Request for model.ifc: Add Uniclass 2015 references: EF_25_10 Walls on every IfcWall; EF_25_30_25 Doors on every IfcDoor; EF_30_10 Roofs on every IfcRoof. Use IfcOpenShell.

First a look at what the model holds.

```python
import ifcopenshell

model = ifcopenshell.open("model.ifc")
print(model.schema)
print("classifications:", [c.Name for c in model.by_type("IfcClassification")])
for ifc_class in ("IfcDoor", "IfcRoof", "IfcStair", "IfcWall", "IfcWindow"):
    print(ifc_class, len(model.by_type(ifc_class)))
```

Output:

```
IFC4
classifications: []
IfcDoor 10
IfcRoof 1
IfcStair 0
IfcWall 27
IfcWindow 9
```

```python
import ifcopenshell
import ifcopenshell.api.classification

model = ifcopenshell.open("model.ifc")

system = ifcopenshell.api.classification.add_classification(model, classification="Uniclass 2015")

codes = {
    "IfcWall": ("EF_25_10", "Walls"),
    "IfcDoor": ("EF_25_30_25", "Doors"),
    "IfcRoof": ("EF_30_10", "Roofs"),
}
for ifc_class, (code, name) in codes.items():
    products = model.by_type(ifc_class)
    ifcopenshell.api.classification.add_reference(
        model, products=products, classification=system, identification=code, name=name
    )
    print(code, len(products))

model.write("model_edited.ifc")
```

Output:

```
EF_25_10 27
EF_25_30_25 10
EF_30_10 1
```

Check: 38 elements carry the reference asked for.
